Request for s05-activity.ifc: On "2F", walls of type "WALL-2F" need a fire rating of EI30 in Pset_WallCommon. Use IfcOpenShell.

First a look at what the model holds.

```python
import ifcopenshell
import ifcopenshell.util.element

model = ifcopenshell.open("s05-activity.ifc")
print(model.schema)
storey = next(s for s in model.by_type("IfcBuildingStorey") if s.Name == "2F")
walls = [e for e in ifcopenshell.util.element.get_decomposition(storey) if e.is_a("IfcWall")]
seen = {}
for e in walls:
    element_type = ifcopenshell.util.element.get_type(e)
    key = (element_type.Name if element_type != e and element_type else None, ifcopenshell.util.element.get_pset(e, "Pset_WallCommon", "FireRating"))
    seen[key] = seen.get(key, 0) + 1
for (name, value), count in sorted(seen.items(), key=str):
    print(count, "x", name, "|", value)
```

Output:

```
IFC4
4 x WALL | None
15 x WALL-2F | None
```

```python
import ifcopenshell
import ifcopenshell.api.pset
import ifcopenshell.util.element

model = ifcopenshell.open("s05-activity.ifc")

storey = next(s for s in model.by_type("IfcBuildingStorey") if s.Name == "2F")
walls = [e for e in ifcopenshell.util.element.get_decomposition(storey) if e.is_a("IfcWall")]

count = 0
for e in walls:
    element_type = ifcopenshell.util.element.get_type(e)
    if element_type in (None, e) or element_type.Name != "WALL-2F":
        continue
    # add_pset returns the element's existing set when there is one.
    pset = ifcopenshell.api.pset.add_pset(model, product=e, name="Pset_WallCommon")
    ifcopenshell.api.pset.edit_pset(model, pset=pset, properties={"FireRating": "EI30"})
    count += 1

print(count, "walls updated")

model.write("s05-activity_v2.ifc")
```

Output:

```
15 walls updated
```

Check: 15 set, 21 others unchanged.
